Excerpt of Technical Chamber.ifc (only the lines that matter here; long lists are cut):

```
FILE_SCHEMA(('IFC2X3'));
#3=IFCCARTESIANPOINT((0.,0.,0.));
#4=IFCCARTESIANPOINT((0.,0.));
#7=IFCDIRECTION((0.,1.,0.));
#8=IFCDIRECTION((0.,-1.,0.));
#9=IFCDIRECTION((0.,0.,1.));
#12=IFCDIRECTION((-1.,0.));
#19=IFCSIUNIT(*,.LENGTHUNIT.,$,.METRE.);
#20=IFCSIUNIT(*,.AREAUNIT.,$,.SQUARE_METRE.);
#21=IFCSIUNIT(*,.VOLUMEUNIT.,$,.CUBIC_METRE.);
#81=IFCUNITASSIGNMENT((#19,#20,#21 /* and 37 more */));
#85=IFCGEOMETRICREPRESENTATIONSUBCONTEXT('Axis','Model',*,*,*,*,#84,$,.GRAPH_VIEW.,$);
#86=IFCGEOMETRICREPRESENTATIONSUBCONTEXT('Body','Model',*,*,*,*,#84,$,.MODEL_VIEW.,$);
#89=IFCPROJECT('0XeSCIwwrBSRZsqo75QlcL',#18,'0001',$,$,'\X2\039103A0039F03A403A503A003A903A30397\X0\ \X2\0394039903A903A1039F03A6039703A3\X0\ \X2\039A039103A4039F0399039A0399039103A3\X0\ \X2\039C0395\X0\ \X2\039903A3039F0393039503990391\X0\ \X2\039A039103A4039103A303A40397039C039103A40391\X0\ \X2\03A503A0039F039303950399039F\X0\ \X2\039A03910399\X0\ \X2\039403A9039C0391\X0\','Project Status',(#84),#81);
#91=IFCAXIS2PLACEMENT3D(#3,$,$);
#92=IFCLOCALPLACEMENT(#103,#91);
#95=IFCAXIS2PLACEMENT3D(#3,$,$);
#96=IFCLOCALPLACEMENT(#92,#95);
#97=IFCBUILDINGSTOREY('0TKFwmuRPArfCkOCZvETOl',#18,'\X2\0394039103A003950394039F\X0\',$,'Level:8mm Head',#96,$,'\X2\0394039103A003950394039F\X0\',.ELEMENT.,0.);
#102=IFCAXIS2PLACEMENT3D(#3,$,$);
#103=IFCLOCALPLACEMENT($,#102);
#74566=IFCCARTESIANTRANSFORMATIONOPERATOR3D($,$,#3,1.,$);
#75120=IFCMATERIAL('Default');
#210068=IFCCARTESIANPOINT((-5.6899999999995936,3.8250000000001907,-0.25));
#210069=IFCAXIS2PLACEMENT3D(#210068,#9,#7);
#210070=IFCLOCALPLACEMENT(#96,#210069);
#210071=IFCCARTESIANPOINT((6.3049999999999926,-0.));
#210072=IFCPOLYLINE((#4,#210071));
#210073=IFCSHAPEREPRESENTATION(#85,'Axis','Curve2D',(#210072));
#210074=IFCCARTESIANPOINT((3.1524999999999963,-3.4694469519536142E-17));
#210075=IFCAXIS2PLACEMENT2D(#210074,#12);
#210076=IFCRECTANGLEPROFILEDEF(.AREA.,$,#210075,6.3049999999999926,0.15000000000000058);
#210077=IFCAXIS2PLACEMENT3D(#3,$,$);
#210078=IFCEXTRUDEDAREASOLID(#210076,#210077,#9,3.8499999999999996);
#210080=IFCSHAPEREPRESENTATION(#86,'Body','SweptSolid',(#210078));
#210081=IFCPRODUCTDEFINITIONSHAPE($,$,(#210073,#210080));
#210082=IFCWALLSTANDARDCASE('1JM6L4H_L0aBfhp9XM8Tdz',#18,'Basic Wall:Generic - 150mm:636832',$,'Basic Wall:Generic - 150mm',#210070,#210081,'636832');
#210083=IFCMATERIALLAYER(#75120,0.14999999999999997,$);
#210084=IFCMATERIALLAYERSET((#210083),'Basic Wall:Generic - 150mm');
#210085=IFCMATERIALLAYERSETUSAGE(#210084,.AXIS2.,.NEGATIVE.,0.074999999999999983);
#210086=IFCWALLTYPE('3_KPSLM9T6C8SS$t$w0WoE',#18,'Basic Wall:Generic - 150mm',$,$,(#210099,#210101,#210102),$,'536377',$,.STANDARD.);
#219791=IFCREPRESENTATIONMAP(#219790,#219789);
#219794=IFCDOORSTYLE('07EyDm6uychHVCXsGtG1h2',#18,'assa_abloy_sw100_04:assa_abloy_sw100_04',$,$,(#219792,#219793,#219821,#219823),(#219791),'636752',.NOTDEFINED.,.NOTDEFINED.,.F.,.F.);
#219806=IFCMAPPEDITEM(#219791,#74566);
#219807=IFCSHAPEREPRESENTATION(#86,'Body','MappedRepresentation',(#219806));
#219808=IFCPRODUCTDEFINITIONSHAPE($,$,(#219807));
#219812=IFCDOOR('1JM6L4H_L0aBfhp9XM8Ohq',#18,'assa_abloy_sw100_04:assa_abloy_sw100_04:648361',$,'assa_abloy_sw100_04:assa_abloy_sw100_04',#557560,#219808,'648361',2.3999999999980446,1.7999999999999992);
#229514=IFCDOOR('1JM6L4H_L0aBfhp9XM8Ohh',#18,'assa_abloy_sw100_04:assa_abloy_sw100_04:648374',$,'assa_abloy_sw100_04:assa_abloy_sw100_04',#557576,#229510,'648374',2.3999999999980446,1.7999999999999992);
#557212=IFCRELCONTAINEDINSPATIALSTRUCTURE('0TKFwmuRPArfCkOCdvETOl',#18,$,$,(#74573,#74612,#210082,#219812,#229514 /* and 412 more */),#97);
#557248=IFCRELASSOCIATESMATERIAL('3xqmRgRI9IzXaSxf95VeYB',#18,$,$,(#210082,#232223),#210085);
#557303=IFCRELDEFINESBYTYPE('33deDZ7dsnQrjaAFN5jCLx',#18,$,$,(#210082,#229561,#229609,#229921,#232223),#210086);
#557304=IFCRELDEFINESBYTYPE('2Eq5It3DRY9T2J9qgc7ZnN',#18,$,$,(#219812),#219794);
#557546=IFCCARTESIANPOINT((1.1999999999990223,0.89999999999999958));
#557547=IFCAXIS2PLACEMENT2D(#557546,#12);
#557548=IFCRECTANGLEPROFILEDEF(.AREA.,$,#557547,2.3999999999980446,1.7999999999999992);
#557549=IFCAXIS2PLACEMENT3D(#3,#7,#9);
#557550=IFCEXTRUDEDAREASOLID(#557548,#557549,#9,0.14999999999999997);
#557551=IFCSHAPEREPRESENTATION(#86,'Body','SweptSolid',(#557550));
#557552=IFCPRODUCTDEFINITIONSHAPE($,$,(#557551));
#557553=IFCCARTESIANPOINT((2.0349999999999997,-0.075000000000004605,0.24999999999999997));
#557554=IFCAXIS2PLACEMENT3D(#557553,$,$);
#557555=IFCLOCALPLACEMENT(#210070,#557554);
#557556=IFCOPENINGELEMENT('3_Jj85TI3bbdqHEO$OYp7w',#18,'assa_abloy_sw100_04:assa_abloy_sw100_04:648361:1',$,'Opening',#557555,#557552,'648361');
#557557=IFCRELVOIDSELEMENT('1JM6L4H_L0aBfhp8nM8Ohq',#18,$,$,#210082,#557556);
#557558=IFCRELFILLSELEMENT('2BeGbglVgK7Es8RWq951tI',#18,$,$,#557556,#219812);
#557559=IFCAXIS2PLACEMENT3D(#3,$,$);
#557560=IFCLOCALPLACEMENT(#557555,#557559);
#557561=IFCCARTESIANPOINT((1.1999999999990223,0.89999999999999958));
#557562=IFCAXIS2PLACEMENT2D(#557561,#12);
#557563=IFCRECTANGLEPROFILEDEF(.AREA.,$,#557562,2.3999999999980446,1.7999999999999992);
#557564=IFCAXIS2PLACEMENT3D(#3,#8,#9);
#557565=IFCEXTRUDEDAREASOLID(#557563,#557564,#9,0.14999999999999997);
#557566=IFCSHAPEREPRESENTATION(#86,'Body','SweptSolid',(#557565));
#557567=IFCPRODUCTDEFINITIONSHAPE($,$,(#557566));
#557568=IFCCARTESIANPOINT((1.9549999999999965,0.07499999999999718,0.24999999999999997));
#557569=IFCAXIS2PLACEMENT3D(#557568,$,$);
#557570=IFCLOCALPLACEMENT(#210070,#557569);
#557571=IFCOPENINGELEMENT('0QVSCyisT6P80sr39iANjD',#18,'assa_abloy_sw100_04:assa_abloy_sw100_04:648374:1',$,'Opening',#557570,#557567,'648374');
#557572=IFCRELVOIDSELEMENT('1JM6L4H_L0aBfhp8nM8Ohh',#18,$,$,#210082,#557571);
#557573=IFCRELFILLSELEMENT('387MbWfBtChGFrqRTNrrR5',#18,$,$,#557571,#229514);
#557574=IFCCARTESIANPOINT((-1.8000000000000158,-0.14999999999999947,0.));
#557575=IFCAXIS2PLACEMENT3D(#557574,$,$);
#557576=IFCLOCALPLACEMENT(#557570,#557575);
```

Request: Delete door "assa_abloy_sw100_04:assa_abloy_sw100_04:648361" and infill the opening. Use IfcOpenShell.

```python
import ifcopenshell
import ifcopenshell.api.feature
import ifcopenshell.api.root
import ifcopenshell.geom
import ifcopenshell.util.shape

model = ifcopenshell.open("Technical Chamber.ifc")
settings = ifcopenshell.geom.settings()


def volume(element):
    """Net volume in cubic metres, openings subtracted."""
    shape = ifcopenshell.geom.create_shape(settings, element)
    return ifcopenshell.util.shape.get_volume(shape.geometry)


door = model.by_guid("1JM6L4H_L0aBfhp9XM8Ohq")
opening = door.FillsVoids[0].RelatingOpeningElement
wall = opening.VoidsElements[0].RelatingBuildingElement
before = volume(wall)

ifcopenshell.api.root.remove_product(model, product=door)
ifcopenshell.api.feature.remove_feature(model, feature=opening)

after = volume(wall)

print(f"wall volume {before:.3f} -> {after:.3f} m3")

model.write("Technical Chamber_updated.ifc")
```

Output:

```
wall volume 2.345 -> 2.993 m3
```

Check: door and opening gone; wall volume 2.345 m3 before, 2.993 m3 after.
